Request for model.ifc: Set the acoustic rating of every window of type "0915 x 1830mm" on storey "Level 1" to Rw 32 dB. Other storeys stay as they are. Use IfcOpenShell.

First a look at what the model holds.

```python
import ifcopenshell
import ifcopenshell.util.element

model = ifcopenshell.open("model.ifc")
print(model.schema)
storey = next(s for s in model.by_type("IfcBuildingStorey") if s.Name == "Level 1")
windows = [e for e in ifcopenshell.util.element.get_decomposition(storey) if e.is_a("IfcWindow")]
seen = {}
for e in windows:
    element_type = ifcopenshell.util.element.get_type(e)
    key = (element_type.Name if element_type != e and element_type else None, ifcopenshell.util.element.get_pset(e, "Pset_WindowCommon", "AcousticRating"))
    seen[key] = seen.get(key, 0) + 1
for (name, value), count in sorted(seen.items(), key=str):
    print(count, "x", name, "|", value)
```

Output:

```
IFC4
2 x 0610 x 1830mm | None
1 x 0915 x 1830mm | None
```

```python
import ifcopenshell
import ifcopenshell.api.pset
import ifcopenshell.util.element

model = ifcopenshell.open("model.ifc")

storey = next(s for s in model.by_type("IfcBuildingStorey") if s.Name == "Level 1")
windows = [e for e in ifcopenshell.util.element.get_decomposition(storey) if e.is_a("IfcWindow")]

count = 0
for e in windows:
    element_type = ifcopenshell.util.element.get_type(e)
    if element_type in (None, e) or element_type.Name != "0915 x 1830mm":
        continue
    # add_pset returns the element's existing set when there is one.
    pset = ifcopenshell.api.pset.add_pset(model, product=e, name="Pset_WindowCommon")
    ifcopenshell.api.pset.edit_pset(model, pset=pset, properties={"AcousticRating": "Rw 32 dB"})
    count += 1

print(count, "windows updated")

model.write("model_edited.ifc")
```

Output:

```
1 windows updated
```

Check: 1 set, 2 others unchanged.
